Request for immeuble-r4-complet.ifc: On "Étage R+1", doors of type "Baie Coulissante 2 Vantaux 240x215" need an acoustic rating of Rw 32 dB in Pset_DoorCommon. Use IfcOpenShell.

First a look at what the model holds.

```python
import ifcopenshell
import ifcopenshell.util.element

model = ifcopenshell.open("immeuble-r4-complet.ifc")
print(model.schema)
storey = next(s for s in model.by_type("IfcBuildingStorey") if s.Name == "Étage R+1")
doors = [e for e in ifcopenshell.util.element.get_decomposition(storey) if e.is_a("IfcDoor")]
seen = {}
for e in doors:
    element_type = ifcopenshell.util.element.get_type(e)
    key = (element_type.Name if element_type != e and element_type else None, ifcopenshell.util.element.get_pset(e, "Pset_DoorCommon", "AcousticRating"))
    seen[key] = seen.get(key, 0) + 1
for (name, value), count in sorted(seen.items(), key=str):
    print(count, "x", name, "|", value)
```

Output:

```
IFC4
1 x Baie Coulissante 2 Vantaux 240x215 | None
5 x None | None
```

```python
import ifcopenshell
import ifcopenshell.api.pset
import ifcopenshell.util.element

model = ifcopenshell.open("immeuble-r4-complet.ifc")

storey = next(s for s in model.by_type("IfcBuildingStorey") if s.Name == "Étage R+1")
doors = [e for e in ifcopenshell.util.element.get_decomposition(storey) if e.is_a("IfcDoor")]

count = 0
for e in doors:
    element_type = ifcopenshell.util.element.get_type(e)
    if element_type in (None, e) or element_type.Name != "Baie Coulissante 2 Vantaux 240x215":
        continue
    # add_pset returns the element's existing set when there is one.
    pset = ifcopenshell.api.pset.add_pset(model, product=e, name="Pset_DoorCommon")
    ifcopenshell.api.pset.edit_pset(model, pset=pset, properties={"AcousticRating": "Rw 32 dB"})
    count += 1

print(count, "doors updated")

model.write("immeuble-r4-complet-out.ifc")
```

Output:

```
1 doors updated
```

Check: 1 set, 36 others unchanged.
